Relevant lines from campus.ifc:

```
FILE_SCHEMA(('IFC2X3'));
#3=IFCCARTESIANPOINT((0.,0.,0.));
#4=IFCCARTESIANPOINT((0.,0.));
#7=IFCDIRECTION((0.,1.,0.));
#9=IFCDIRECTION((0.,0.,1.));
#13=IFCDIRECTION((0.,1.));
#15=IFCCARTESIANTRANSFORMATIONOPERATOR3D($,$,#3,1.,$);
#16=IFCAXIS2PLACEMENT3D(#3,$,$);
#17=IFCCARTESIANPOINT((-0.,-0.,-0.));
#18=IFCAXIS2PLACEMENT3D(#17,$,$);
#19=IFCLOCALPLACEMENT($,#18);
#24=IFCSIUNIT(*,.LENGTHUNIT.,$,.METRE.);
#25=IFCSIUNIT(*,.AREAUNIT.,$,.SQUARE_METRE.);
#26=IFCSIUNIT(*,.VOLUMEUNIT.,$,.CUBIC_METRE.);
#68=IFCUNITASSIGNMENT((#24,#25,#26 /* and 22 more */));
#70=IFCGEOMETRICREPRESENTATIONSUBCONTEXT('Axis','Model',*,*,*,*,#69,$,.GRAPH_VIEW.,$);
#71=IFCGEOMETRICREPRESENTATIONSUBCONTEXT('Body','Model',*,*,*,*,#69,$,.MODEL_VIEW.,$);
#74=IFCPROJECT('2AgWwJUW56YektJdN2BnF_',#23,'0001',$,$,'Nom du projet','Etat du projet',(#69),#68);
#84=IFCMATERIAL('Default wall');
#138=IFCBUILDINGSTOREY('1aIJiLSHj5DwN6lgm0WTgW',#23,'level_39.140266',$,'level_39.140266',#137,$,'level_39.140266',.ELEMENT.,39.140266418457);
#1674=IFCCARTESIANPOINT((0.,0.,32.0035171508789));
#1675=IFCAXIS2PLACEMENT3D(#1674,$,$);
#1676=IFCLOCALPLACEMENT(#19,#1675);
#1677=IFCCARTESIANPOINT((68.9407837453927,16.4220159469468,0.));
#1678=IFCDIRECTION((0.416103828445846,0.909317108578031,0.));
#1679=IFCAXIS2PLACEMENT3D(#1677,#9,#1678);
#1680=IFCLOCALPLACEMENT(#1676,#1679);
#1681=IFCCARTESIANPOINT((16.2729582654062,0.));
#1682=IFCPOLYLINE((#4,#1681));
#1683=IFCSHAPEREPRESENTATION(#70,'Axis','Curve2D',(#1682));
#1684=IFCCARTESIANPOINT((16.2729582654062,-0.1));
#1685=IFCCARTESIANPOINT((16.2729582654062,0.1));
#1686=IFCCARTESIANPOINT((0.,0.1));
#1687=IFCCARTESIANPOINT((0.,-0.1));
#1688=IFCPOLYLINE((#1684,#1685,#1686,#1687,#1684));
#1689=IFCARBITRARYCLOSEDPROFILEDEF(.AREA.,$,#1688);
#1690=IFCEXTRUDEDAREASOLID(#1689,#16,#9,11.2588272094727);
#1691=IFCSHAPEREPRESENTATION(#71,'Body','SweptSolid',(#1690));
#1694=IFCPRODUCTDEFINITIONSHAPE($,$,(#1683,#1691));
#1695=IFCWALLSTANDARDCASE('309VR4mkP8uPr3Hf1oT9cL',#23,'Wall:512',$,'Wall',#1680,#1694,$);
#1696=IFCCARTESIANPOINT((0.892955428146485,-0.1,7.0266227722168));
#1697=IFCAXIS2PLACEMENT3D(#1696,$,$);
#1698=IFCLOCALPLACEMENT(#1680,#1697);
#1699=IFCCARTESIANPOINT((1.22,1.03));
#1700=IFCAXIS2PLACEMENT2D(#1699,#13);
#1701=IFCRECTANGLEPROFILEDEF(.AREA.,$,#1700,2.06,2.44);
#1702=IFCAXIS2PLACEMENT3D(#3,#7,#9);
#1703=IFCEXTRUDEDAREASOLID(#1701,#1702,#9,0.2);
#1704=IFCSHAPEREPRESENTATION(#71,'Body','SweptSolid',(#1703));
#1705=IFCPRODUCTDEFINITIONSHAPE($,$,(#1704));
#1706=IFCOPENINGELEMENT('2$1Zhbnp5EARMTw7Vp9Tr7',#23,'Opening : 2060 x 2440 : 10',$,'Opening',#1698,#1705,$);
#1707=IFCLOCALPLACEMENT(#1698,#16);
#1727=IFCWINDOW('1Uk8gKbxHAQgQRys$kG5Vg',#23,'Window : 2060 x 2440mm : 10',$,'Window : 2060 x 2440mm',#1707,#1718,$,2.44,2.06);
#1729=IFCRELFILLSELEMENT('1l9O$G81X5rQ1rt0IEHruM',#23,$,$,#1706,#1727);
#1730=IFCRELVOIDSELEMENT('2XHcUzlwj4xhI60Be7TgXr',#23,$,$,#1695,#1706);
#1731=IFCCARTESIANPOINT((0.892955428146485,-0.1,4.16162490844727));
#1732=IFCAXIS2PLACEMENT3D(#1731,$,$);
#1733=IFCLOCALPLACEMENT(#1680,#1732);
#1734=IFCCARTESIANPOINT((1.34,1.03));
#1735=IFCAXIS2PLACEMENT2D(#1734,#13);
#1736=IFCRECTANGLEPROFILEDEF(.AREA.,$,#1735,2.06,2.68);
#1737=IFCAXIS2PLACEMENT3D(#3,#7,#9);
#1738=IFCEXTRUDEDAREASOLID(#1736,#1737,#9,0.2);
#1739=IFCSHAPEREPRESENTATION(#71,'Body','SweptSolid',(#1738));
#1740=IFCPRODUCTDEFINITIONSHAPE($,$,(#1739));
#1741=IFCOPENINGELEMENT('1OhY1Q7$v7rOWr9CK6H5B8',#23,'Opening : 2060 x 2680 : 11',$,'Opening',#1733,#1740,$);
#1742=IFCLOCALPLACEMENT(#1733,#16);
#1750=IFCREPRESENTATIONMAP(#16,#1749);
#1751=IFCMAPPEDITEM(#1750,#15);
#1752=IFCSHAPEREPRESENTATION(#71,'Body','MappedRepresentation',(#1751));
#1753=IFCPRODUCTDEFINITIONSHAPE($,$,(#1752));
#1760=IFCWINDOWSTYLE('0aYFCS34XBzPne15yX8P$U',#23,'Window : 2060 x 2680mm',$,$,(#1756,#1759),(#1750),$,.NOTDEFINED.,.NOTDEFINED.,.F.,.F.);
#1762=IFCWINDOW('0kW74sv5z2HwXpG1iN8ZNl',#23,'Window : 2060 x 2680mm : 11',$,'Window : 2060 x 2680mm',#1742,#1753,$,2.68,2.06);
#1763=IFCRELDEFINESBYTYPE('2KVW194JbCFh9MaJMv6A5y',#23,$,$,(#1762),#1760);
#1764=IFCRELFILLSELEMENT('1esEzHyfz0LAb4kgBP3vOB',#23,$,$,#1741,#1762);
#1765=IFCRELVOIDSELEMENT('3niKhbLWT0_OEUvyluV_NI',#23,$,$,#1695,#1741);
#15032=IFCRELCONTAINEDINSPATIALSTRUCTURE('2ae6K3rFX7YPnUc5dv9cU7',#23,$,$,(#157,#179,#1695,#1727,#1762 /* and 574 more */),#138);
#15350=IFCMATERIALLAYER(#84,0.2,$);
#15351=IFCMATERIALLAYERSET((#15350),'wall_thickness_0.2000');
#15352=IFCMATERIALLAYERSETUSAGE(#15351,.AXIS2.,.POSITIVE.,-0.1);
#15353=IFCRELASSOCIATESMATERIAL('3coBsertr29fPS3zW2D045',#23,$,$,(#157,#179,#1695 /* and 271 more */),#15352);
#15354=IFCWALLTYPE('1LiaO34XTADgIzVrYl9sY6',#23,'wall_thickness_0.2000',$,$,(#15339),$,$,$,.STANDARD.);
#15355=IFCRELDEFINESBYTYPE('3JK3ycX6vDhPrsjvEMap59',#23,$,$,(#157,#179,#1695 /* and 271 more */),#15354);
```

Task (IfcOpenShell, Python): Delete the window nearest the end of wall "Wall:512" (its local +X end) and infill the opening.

```python
import ifcopenshell
import ifcopenshell.api.feature
import ifcopenshell.api.root
import ifcopenshell.geom
import ifcopenshell.util.shape

model = ifcopenshell.open("campus.ifc")
settings = ifcopenshell.geom.settings()


def volume(element):
    """Net volume in cubic metres, openings subtracted."""
    shape = ifcopenshell.geom.create_shape(settings, element)
    return ifcopenshell.util.shape.get_volume(shape.geometry)


window = model.by_id(1762)
opening = window.FillsVoids[0].RelatingOpeningElement
wall = opening.VoidsElements[0].RelatingBuildingElement
before = volume(wall)

ifcopenshell.api.root.remove_product(model, product=window)
ifcopenshell.api.feature.remove_feature(model, feature=opening)

after = volume(wall)

print(f"wall volume {before:.3f} -> {after:.3f} m3")

model.write("campus_edited.ifc")
```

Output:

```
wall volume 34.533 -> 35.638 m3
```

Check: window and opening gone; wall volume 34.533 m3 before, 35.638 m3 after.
